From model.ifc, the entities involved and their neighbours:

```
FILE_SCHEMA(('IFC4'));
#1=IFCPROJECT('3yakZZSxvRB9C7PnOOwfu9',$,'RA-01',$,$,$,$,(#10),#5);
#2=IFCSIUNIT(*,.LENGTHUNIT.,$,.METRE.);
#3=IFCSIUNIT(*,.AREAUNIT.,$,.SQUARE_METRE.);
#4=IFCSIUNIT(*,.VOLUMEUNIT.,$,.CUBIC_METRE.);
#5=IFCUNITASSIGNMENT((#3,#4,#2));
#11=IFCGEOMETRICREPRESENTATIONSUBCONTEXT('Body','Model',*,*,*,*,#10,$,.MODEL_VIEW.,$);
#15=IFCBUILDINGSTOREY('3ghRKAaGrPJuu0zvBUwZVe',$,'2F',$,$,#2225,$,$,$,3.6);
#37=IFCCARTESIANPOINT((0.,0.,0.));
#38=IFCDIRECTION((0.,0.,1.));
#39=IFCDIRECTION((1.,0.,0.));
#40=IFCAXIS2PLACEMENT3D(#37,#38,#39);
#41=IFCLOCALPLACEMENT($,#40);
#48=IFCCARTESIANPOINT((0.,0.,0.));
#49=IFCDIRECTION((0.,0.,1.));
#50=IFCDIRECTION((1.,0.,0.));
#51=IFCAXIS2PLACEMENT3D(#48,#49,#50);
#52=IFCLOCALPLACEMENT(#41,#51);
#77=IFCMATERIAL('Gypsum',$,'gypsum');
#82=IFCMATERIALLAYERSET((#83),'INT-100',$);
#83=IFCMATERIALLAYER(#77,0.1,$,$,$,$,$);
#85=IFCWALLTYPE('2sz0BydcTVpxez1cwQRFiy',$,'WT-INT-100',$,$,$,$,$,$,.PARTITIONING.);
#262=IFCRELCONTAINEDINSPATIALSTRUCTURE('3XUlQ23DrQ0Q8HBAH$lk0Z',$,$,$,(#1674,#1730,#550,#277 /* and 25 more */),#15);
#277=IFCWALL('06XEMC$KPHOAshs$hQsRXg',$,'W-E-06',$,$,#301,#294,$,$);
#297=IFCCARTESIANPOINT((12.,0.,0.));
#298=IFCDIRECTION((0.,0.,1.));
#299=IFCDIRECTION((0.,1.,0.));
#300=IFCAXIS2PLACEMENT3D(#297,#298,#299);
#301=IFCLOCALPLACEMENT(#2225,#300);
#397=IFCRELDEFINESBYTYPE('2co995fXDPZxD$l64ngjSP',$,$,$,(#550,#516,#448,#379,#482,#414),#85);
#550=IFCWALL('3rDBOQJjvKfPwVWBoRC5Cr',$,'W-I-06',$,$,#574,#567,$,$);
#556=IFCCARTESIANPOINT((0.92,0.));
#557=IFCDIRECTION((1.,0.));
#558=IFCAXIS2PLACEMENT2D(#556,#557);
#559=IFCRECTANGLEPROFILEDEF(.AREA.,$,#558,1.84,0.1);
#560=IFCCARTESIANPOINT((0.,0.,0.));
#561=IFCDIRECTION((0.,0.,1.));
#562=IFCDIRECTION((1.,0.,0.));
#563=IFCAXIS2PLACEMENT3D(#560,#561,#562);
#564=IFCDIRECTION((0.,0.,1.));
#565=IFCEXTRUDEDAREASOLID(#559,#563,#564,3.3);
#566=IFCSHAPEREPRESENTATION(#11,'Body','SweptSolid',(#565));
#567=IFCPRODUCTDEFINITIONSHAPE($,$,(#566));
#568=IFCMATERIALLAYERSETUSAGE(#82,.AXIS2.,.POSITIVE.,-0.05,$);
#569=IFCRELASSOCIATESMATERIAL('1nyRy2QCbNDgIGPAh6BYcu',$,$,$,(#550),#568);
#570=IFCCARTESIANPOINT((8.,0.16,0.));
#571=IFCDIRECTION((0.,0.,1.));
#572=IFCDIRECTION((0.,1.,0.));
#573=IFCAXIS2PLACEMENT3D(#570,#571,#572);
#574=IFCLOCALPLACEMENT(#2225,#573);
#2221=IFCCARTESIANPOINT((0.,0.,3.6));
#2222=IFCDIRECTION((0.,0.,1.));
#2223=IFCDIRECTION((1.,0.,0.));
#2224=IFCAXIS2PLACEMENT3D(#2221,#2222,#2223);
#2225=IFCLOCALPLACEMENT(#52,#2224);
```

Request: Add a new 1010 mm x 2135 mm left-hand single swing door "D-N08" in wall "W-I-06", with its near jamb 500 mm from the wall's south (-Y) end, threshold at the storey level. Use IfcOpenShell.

```python
import numpy as np
import ifcopenshell
import ifcopenshell.api.feature
import ifcopenshell.api.geometry
import ifcopenshell.api.root
import ifcopenshell.api.spatial
import ifcopenshell.geom
import ifcopenshell.util.element
import ifcopenshell.util.placement
import ifcopenshell.util.representation
import ifcopenshell.util.shape
import ifcopenshell.util.unit

model = ifcopenshell.open("model.ifc")
unit_scale = ifcopenshell.util.unit.calculate_unit_scale(model)
settings = ifcopenshell.geom.settings()


def volume(element):
    """Net volume in cubic metres, openings subtracted."""
    shape = ifcopenshell.geom.create_shape(settings, element)
    return ifcopenshell.util.shape.get_volume(shape.geometry)


wall = model.by_id(550)
storey = ifcopenshell.util.element.get_container(wall, ifc_class="IfcBuildingStorey")
context = ifcopenshell.util.representation.get_context(model, "Model", "Body", "MODEL_VIEW")
before = volume(wall)

width, height, from_end, sill = 1.01, 2.135, 0.5, 0.0  # metres

# The wall runs along its own X axis, and the end named is its -X end.
wall_shape = ifcopenshell.geom.create_shape(settings, wall)
x, y, z = ifcopenshell.util.shape.get_vertices(wall_shape.geometry).T
start = x.min() + from_end
face, thickness = float(y.min()), float(y.max() - y.min())
wall_matrix = ifcopenshell.util.placement.get_local_placement(wall.ObjectPlacement)
level = ifcopenshell.util.placement.get_local_placement(storey.ObjectPlacement)[2, 3]


def in_wall(x, y):
    """Placement at x, y metres in the wall's axes, at sill height."""
    matrix = wall_matrix.copy()
    matrix[:, 3] = wall_matrix @ np.array([x / unit_scale, y / unit_scale, 0.0, 1.0])
    matrix[2, 3] = level + sill / unit_scale
    return matrix


# Opening: a box that overshoots both wall faces by 50 mm.
opening = ifcopenshell.api.root.create_entity(model, ifc_class="IfcOpeningElement", predefined_type="OPENING")
box = ifcopenshell.api.geometry.add_wall_representation(
    model, context=context, length=width, height=height, thickness=thickness + 0.1
)
ifcopenshell.api.geometry.assign_representation(model, product=opening, representation=box)
ifcopenshell.api.geometry.edit_object_placement(model, product=opening, matrix=in_wall(start, face - 0.05), is_si=False)
ifcopenshell.api.feature.add_feature(model, feature=opening, element=wall)

door = ifcopenshell.api.root.create_entity(model, ifc_class="IfcDoor", name="D-N08", predefined_type="DOOR")
door.OverallWidth, door.OverallHeight = width / unit_scale, height / unit_scale
door.OperationType = "SINGLE_SWING_LEFT"
body = ifcopenshell.api.geometry.add_door_representation(
    model,
    context=context,
    overall_width=door.OverallWidth,
    overall_height=door.OverallHeight,
    operation_type="SINGLE_SWING_LEFT",
    lining_properties={"LiningDepth": thickness / unit_scale, "ThresholdDepth": thickness / unit_scale},
)
ifcopenshell.api.geometry.assign_representation(model, product=door, representation=body)
ifcopenshell.api.spatial.assign_container(model, products=[door], relating_structure=storey)
ifcopenshell.api.feature.add_filling(model, opening=opening, element=door)

# The lining spans the wall, so the door starts at the wall face.
ifcopenshell.api.geometry.edit_object_placement(model, product=door, matrix=in_wall(start, face), is_si=False)

after = volume(wall)

print(f"wall volume {before:.3f} -> {after:.3f} m3")

model.write("model_updated.ifc")
```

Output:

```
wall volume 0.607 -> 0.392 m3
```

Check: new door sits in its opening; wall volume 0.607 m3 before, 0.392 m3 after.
